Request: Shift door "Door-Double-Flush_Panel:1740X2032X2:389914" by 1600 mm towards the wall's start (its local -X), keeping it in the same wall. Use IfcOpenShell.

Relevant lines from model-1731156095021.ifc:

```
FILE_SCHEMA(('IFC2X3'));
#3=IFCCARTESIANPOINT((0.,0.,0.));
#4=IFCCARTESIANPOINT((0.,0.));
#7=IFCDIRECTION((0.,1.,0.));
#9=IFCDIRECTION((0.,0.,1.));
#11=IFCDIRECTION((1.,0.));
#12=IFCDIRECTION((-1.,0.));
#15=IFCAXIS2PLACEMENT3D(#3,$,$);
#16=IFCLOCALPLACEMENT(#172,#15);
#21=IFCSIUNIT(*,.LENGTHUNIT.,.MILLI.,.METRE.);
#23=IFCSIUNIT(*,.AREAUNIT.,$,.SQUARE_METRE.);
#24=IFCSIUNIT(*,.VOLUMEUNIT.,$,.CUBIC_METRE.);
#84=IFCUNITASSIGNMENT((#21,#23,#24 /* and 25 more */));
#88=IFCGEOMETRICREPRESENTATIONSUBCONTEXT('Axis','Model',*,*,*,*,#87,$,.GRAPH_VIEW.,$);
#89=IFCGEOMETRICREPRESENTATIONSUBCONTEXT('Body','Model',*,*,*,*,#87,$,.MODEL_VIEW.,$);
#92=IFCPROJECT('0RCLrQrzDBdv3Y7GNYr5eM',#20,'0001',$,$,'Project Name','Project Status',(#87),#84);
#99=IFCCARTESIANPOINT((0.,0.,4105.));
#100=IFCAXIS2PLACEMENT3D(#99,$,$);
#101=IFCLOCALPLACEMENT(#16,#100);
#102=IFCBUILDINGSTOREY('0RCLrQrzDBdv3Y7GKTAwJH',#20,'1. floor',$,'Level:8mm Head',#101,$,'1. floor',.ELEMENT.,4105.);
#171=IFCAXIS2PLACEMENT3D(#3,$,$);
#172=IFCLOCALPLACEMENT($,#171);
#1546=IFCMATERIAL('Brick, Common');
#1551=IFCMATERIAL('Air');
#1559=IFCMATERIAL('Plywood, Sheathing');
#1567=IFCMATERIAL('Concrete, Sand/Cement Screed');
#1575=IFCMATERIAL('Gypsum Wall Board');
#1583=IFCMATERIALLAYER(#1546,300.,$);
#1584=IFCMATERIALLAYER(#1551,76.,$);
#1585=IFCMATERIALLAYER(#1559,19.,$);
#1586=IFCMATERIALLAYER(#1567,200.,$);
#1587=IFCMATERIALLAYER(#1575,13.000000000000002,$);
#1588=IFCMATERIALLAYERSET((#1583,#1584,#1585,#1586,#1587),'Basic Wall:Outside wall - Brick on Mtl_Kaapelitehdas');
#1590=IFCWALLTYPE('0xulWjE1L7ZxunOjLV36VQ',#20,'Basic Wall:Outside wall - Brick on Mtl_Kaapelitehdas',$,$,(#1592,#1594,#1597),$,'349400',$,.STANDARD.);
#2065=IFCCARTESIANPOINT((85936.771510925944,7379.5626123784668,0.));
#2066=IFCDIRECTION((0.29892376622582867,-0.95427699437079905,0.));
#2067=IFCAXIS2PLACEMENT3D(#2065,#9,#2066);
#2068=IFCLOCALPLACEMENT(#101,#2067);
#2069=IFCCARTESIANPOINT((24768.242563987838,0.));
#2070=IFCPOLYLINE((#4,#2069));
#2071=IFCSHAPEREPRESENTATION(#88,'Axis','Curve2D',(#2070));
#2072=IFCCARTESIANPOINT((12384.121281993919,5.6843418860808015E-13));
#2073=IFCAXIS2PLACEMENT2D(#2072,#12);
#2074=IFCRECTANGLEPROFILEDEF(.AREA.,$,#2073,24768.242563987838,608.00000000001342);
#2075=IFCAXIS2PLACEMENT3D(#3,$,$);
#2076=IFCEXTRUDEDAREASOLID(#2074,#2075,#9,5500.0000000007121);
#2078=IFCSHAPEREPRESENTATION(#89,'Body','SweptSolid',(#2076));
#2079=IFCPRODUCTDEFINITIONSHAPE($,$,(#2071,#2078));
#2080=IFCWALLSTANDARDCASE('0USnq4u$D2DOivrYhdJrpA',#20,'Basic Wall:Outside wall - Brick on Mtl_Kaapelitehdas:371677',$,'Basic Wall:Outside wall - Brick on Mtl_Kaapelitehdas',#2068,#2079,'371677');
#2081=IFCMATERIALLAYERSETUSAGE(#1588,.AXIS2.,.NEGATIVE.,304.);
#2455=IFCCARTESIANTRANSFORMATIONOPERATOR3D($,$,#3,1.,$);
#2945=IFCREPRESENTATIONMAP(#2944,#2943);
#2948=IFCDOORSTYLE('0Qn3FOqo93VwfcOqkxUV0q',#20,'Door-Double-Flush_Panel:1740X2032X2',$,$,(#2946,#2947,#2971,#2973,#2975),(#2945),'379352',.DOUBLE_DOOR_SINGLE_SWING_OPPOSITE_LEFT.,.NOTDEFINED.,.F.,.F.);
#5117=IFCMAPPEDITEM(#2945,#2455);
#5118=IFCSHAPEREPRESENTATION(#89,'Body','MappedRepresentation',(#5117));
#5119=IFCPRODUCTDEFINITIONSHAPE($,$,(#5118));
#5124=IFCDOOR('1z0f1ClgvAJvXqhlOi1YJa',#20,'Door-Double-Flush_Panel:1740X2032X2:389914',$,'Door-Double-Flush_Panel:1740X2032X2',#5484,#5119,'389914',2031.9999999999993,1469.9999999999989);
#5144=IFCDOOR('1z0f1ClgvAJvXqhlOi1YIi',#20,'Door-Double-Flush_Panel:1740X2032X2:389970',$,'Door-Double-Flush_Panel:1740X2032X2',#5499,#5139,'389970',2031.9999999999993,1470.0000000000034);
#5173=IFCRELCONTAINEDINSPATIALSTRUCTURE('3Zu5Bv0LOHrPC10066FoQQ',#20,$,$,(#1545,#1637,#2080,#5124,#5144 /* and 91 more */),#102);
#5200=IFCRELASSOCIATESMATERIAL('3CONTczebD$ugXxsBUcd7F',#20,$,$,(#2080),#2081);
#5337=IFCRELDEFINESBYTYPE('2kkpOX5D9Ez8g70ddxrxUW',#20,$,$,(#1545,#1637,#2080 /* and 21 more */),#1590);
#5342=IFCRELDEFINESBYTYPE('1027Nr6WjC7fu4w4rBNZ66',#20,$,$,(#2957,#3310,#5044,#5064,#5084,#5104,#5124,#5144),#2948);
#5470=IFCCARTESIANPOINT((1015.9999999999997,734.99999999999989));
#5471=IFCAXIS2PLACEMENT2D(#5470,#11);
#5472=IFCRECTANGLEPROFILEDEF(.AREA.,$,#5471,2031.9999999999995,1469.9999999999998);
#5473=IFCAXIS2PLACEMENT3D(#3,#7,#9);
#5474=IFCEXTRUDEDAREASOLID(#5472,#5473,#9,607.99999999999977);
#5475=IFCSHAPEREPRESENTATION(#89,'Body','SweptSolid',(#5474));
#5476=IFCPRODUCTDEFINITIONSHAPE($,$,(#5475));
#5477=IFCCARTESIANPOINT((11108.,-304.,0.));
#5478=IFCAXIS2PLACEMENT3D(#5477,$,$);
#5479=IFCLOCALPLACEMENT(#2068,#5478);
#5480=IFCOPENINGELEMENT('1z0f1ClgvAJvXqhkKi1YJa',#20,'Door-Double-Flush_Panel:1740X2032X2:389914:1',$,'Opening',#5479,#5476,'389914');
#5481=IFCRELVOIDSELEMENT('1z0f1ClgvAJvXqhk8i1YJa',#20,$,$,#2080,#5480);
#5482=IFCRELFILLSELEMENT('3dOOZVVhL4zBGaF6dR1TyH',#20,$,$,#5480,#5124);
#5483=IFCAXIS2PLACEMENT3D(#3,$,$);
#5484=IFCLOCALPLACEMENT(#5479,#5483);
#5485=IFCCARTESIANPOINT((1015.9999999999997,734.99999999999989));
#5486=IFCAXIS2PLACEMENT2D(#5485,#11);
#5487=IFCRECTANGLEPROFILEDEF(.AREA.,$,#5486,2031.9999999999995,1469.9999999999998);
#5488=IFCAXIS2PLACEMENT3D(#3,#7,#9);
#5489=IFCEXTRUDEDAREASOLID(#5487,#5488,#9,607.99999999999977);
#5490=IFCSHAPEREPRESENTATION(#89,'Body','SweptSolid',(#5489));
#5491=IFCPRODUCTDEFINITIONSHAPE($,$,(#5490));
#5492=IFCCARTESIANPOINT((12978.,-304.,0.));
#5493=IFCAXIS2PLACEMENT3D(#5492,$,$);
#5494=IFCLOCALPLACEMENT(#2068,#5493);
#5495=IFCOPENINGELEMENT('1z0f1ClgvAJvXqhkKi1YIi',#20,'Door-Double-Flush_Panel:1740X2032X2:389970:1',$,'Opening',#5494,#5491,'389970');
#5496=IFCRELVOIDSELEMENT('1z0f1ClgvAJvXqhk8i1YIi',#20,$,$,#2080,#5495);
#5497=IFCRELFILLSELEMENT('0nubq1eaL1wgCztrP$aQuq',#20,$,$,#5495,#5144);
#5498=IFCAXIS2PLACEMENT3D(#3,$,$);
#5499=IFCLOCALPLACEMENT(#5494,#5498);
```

```python
import ifcopenshell
import ifcopenshell.api.geometry
import ifcopenshell.util.placement
import ifcopenshell.util.unit

model = ifcopenshell.open("model-1731156095021.ifc")
unit_scale = ifcopenshell.util.unit.calculate_unit_scale(model)

door = model.by_guid("1z0f1ClgvAJvXqhlOi1YJa")
opening = door.FillsVoids[0].RelatingOpeningElement
wall = opening.VoidsElements[0].RelatingBuildingElement

wall_matrix = ifcopenshell.util.placement.get_local_placement(wall.ObjectPlacement)
shift = wall_matrix[:3, 0] * -1.6 / unit_scale
before = ifcopenshell.util.placement.get_local_placement(door.ObjectPlacement)[:3, 3].copy()

# The door is placed relative to its opening, so it follows when the opening moves.
matrix = ifcopenshell.util.placement.get_local_placement(opening.ObjectPlacement)
matrix[:3, 3] += shift
ifcopenshell.api.geometry.edit_object_placement(
    model, product=opening, matrix=matrix, is_si=False, should_transform_children=True
)

after = ifcopenshell.util.placement.get_local_placement(door.ObjectPlacement)[:3, 3]
print("door moved by", (after - before).round(3) + 0.0)

model.write("model-1731156095021_updated.ifc")
```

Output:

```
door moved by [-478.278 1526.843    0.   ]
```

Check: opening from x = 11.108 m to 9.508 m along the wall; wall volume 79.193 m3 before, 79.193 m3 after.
